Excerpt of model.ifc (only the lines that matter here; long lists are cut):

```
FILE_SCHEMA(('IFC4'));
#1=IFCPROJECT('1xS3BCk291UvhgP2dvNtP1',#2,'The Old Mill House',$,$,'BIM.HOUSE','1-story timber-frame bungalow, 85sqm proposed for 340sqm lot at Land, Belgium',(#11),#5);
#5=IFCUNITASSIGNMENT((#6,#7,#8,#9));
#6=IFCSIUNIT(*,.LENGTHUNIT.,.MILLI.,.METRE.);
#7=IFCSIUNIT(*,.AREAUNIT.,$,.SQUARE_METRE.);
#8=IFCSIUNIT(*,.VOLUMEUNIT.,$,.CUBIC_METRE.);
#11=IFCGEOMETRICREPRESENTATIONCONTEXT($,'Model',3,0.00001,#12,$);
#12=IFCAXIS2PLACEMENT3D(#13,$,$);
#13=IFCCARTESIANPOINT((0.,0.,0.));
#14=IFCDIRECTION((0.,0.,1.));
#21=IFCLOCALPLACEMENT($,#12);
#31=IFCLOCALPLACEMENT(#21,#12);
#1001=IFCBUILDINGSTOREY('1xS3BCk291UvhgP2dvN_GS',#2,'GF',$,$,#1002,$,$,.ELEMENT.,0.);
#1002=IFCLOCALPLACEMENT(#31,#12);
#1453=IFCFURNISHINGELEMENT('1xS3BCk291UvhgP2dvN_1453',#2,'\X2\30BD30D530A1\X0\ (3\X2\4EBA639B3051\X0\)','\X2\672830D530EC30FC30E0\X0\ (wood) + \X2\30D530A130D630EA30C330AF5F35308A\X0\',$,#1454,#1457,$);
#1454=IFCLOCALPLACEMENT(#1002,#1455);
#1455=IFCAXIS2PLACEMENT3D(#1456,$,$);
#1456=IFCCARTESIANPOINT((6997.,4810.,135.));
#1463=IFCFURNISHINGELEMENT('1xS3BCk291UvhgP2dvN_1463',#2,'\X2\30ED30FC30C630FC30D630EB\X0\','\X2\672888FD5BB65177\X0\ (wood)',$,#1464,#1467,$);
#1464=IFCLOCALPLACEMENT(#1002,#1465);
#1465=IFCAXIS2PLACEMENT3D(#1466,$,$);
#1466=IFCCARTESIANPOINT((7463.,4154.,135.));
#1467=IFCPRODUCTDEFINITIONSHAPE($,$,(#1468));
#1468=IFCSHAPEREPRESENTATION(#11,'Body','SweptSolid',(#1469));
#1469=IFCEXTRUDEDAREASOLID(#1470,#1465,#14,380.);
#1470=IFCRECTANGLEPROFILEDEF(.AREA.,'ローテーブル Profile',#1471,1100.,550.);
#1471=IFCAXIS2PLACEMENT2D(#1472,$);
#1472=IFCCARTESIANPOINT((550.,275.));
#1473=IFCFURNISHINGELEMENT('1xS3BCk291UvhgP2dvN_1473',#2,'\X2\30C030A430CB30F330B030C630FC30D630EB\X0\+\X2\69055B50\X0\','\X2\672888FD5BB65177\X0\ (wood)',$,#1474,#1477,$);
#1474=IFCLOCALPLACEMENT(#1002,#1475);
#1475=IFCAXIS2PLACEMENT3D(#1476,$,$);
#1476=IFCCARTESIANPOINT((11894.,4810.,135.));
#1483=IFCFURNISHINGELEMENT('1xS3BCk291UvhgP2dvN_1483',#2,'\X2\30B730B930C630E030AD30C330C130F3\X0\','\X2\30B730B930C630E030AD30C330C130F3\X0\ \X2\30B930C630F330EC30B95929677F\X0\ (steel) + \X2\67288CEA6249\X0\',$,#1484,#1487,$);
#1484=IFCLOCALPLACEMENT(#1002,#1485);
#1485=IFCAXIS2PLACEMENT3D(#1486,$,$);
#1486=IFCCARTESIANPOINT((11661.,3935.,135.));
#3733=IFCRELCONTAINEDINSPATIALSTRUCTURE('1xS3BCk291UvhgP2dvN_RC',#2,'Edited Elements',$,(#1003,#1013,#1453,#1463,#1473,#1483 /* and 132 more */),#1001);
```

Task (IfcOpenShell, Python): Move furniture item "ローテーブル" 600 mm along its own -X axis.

```python
import ifcopenshell
import ifcopenshell.api.geometry
import ifcopenshell.util.placement

model = ifcopenshell.open("model.ifc")

item = model.by_guid("1xS3BCk291UvhgP2dvN_1463")
matrix = ifcopenshell.util.placement.get_local_placement(item.ObjectPlacement)
matrix[:3, 3] -= matrix[:3, 0] * 600.0
ifcopenshell.api.geometry.edit_object_placement(model, product=item, matrix=matrix, is_si=False)

print(ifcopenshell.util.placement.get_local_placement(item.ObjectPlacement).round(3) + 0.0)

model.write("model_updated.ifc")
```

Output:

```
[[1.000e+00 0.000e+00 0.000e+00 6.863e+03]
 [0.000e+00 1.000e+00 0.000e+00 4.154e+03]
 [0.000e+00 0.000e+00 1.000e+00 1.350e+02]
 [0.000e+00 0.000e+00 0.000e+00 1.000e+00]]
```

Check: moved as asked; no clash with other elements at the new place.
